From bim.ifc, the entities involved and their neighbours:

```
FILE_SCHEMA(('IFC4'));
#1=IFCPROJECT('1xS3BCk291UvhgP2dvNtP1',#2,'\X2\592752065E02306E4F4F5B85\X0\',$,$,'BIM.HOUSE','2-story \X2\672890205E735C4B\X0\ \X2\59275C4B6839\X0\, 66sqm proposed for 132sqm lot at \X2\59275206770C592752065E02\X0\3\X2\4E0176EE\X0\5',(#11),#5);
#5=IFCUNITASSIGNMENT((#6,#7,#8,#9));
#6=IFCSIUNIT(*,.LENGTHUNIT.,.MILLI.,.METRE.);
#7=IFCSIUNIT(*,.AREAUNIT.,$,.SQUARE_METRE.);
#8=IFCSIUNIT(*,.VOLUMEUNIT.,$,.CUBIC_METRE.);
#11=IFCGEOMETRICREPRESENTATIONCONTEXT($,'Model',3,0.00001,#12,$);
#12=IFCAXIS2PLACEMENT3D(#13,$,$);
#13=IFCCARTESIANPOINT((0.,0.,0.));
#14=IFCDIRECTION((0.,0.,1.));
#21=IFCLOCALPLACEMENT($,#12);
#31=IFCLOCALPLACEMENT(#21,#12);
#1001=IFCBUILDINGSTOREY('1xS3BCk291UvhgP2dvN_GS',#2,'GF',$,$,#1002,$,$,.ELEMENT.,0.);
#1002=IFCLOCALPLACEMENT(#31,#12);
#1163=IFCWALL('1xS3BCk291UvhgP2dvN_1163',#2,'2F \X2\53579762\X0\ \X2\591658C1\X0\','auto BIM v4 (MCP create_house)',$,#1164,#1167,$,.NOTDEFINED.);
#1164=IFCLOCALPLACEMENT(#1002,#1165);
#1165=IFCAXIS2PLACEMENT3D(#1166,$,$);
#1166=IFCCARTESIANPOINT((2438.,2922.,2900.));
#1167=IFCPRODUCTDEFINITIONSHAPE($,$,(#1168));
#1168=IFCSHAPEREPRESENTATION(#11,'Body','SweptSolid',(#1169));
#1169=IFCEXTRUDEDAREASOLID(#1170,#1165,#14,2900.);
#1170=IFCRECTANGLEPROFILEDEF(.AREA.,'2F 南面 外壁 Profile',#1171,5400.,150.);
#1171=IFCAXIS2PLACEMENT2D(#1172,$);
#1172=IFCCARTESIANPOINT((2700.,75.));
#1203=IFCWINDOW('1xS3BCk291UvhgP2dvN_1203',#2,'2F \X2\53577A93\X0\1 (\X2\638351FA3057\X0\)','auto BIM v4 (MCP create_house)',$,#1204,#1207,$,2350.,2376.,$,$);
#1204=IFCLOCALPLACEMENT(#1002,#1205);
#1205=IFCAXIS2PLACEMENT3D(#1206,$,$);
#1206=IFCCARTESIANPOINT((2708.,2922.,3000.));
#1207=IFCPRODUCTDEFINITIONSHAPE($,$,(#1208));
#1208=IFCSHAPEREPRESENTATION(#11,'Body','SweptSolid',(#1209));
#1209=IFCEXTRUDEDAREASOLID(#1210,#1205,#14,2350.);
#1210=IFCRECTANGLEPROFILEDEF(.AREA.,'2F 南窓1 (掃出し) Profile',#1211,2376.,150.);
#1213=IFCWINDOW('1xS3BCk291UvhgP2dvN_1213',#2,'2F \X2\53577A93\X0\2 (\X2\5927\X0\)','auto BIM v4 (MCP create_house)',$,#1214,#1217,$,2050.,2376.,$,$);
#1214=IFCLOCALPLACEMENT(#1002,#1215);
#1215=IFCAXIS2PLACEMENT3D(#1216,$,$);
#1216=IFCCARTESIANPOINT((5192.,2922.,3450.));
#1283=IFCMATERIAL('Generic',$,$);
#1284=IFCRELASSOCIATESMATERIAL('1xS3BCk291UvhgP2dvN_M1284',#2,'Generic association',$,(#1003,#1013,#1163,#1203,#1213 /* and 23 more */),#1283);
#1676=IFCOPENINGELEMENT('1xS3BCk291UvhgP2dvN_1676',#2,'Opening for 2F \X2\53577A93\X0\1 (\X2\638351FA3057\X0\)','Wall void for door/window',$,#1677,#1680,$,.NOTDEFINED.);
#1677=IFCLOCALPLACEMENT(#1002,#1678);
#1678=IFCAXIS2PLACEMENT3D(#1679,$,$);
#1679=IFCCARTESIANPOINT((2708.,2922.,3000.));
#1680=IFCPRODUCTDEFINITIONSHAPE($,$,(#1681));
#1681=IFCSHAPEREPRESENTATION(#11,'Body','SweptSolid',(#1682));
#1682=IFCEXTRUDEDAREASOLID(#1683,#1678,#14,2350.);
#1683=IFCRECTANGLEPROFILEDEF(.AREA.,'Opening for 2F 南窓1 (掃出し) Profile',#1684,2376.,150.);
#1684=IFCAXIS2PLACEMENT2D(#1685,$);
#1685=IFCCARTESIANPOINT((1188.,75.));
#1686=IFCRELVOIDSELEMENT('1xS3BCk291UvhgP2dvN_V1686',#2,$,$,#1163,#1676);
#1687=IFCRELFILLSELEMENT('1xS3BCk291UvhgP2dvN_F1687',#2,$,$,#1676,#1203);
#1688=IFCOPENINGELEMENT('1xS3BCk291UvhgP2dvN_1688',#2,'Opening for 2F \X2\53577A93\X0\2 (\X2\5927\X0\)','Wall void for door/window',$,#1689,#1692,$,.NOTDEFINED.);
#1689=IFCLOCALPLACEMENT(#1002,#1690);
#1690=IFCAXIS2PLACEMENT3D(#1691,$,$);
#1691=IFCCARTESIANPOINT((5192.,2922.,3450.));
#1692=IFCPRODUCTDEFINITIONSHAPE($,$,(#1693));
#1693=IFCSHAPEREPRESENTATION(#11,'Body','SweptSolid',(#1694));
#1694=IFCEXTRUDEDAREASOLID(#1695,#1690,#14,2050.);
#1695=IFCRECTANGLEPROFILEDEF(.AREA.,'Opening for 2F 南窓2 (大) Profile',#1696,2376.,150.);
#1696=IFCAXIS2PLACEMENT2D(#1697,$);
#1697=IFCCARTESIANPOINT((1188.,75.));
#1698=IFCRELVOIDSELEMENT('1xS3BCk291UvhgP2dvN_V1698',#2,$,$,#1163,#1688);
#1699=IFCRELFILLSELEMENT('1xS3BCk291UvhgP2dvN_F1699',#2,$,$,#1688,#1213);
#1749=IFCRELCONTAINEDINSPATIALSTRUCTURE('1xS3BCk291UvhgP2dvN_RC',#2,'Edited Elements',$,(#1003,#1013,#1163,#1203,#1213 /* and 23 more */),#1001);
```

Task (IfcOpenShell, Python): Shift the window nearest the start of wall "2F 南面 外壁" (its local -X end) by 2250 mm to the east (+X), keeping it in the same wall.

```python
import ifcopenshell
import ifcopenshell.api.geometry
import ifcopenshell.util.placement

model = ifcopenshell.open("bim.ifc")

window = model.by_guid("1xS3BCk291UvhgP2dvN_1203")
opening = window.FillsVoids[0].RelatingOpeningElement
wall = opening.VoidsElements[0].RelatingBuildingElement

wall_matrix = ifcopenshell.util.placement.get_local_placement(wall.ObjectPlacement)
shift = wall_matrix[:3, 0] * 2250.0
before = ifcopenshell.util.placement.get_local_placement(window.ObjectPlacement)[:3, 3].copy()

# The window is not placed relative to its opening, so move both.
for product in (opening, window):
    matrix = ifcopenshell.util.placement.get_local_placement(product.ObjectPlacement)
    matrix[:3, 3] += shift
    ifcopenshell.api.geometry.edit_object_placement(model, product=product, matrix=matrix, is_si=False)

after = ifcopenshell.util.placement.get_local_placement(window.ObjectPlacement)[:3, 3]
print("window moved by", (after - before).round(3) + 0.0)

model.write("bim-out.ifc")
```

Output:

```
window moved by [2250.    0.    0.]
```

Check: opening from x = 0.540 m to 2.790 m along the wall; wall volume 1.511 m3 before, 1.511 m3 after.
